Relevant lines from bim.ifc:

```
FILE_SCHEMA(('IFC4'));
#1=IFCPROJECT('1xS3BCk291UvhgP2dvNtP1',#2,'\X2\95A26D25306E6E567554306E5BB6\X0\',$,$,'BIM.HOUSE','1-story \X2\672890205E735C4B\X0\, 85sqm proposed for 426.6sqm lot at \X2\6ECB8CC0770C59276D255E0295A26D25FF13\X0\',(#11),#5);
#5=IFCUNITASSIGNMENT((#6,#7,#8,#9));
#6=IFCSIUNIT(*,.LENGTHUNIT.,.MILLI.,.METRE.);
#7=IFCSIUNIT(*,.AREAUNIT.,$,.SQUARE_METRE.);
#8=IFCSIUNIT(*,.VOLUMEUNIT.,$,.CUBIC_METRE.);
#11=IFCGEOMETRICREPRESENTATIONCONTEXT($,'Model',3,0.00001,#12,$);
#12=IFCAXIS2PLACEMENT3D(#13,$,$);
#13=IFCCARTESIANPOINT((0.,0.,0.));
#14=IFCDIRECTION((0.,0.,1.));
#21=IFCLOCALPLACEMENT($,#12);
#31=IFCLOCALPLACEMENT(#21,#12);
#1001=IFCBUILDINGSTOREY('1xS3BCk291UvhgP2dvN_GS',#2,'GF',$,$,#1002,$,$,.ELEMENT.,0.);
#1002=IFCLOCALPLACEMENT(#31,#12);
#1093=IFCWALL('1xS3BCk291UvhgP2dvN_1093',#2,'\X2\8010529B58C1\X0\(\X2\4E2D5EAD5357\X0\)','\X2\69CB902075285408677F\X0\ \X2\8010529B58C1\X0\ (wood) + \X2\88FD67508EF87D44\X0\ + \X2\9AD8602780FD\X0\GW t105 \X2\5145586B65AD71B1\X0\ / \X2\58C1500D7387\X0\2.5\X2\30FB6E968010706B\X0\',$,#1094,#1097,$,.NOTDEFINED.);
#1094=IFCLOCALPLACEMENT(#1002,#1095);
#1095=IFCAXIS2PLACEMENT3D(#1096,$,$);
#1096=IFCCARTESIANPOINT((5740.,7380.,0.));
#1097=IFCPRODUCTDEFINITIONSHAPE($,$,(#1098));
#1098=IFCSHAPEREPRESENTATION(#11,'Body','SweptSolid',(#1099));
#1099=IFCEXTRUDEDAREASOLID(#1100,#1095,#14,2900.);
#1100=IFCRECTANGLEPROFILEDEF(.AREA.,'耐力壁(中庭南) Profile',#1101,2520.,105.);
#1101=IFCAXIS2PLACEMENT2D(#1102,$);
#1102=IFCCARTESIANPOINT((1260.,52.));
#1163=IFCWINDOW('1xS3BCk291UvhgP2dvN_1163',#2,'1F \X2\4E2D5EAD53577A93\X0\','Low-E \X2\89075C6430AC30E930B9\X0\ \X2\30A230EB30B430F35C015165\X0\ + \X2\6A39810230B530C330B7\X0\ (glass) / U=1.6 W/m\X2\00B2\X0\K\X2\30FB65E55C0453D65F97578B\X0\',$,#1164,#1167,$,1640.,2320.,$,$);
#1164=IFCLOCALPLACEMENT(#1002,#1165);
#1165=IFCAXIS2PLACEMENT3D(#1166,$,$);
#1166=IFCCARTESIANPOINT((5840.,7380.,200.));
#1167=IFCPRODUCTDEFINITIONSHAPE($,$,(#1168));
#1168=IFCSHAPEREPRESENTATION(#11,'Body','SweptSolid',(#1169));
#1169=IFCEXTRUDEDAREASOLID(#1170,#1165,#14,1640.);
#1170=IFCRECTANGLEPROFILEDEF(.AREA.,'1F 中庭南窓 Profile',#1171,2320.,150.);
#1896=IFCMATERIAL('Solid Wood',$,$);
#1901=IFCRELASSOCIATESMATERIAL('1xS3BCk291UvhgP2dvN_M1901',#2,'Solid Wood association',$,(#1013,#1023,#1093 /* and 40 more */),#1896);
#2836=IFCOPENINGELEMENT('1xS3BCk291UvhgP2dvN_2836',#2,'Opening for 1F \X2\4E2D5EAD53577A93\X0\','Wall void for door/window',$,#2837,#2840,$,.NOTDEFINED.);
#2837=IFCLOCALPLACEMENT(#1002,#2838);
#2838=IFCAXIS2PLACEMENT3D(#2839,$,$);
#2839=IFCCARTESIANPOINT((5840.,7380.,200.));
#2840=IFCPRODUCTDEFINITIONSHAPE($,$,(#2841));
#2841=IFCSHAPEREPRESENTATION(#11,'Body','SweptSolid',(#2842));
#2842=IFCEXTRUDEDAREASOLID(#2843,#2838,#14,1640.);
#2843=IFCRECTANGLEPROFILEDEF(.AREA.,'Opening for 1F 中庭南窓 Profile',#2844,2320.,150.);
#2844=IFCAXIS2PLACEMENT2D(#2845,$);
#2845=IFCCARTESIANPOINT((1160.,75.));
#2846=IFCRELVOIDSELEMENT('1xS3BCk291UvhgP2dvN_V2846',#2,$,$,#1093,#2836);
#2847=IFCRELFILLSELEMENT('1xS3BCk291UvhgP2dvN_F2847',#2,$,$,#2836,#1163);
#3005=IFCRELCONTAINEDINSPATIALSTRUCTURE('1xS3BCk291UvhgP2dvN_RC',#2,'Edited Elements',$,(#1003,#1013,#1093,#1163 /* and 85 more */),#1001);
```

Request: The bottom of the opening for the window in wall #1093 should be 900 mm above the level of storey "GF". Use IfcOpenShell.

```python
import numpy as np
import ifcopenshell
import ifcopenshell.api.geometry
import ifcopenshell.geom
import ifcopenshell.util.element
import ifcopenshell.util.placement
import ifcopenshell.util.shape
import ifcopenshell.util.unit

model = ifcopenshell.open("bim.ifc")
unit_scale = ifcopenshell.util.unit.calculate_unit_scale(model)

window = model.by_id(1163)
opening = window.FillsVoids[0].RelatingOpeningElement
storey = ifcopenshell.util.element.get_container(window, ifc_class="IfcBuildingStorey")
level = ifcopenshell.util.placement.get_local_placement(storey.ObjectPlacement)[2, 3]

# The opening's origin need not be at the sill, so measure its lowest point.
shape = ifcopenshell.geom.create_shape(ifcopenshell.geom.settings(), opening)
bottom = ifcopenshell.util.shape.get_shape_bottom_elevation(shape, shape.geometry) / unit_scale
dz = level + 0.9 / unit_scale - bottom

shift = np.array([0.0, 0.0, dz])
# The window is not placed relative to its opening, so move both.
for product in (opening, window):
    matrix = ifcopenshell.util.placement.get_local_placement(product.ObjectPlacement)
    matrix[:3, 3] += shift
    ifcopenshell.api.geometry.edit_object_placement(model, product=product, matrix=matrix, is_si=False)

print(f"moved by {dz * unit_scale:+.3f} m")

model.write("bim_edited.ifc")
```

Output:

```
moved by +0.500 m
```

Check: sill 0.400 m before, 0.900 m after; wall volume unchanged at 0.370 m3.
